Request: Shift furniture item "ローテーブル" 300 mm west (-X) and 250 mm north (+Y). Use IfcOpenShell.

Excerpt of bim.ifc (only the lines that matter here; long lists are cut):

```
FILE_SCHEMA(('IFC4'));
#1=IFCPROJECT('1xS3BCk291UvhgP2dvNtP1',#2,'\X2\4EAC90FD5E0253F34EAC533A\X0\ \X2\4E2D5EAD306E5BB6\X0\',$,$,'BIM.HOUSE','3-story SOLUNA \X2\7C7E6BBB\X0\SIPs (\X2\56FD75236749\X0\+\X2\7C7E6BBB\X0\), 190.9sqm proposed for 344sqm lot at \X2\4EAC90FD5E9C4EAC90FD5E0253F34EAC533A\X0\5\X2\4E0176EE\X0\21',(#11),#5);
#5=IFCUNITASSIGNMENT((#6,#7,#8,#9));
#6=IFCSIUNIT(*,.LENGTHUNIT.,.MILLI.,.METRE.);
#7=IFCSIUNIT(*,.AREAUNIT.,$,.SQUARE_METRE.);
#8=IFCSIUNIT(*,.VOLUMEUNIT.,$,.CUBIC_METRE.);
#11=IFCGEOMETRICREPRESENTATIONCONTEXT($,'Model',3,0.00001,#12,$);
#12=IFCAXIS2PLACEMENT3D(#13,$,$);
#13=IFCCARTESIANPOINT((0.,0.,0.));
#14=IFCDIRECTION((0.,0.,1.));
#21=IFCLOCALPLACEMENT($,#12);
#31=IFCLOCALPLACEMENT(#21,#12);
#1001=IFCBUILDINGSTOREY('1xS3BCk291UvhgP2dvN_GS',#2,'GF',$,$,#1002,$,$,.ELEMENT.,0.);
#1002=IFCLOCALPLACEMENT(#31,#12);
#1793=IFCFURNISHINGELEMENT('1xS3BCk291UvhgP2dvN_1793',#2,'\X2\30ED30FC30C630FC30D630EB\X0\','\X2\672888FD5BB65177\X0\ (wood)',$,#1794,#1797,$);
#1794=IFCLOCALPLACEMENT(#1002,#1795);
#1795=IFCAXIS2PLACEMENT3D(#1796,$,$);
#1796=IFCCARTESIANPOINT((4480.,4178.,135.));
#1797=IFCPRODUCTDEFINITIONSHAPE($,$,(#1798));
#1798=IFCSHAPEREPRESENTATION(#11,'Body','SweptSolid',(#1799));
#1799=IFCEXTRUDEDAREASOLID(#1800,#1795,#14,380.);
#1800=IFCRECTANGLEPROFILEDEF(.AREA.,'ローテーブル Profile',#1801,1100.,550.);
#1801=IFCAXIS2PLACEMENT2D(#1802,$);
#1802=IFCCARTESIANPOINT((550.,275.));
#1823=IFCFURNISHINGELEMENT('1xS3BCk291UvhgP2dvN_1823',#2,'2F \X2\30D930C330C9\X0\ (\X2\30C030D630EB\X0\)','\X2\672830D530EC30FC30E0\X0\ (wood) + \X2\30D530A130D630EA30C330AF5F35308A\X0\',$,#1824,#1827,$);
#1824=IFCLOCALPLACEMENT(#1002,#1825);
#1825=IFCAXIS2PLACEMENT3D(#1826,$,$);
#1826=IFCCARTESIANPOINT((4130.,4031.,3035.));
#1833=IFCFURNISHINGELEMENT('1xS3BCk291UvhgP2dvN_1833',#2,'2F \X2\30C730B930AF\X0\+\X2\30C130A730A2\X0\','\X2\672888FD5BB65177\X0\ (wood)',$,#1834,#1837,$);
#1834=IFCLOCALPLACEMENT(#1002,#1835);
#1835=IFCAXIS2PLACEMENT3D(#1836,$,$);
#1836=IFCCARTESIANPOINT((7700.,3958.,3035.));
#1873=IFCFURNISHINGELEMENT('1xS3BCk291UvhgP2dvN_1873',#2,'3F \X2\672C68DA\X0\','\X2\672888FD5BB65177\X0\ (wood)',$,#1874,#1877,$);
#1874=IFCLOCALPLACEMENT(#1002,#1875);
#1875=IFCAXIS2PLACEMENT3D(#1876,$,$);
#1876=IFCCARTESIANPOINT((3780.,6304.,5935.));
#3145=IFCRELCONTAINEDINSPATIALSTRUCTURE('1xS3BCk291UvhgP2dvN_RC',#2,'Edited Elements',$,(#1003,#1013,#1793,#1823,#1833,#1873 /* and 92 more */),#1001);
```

```python
import ifcopenshell
import ifcopenshell.api.geometry
import ifcopenshell.util.placement
import ifcopenshell.util.unit

model = ifcopenshell.open("bim.ifc")
unit_scale = ifcopenshell.util.unit.calculate_unit_scale(model)

item = model.by_guid("1xS3BCk291UvhgP2dvN_1793")
matrix = ifcopenshell.util.placement.get_local_placement(item.ObjectPlacement)
matrix[0, 3] -= 0.3 / unit_scale
matrix[1, 3] += 0.25 / unit_scale
ifcopenshell.api.geometry.edit_object_placement(model, product=item, matrix=matrix, is_si=False)

print(ifcopenshell.util.placement.get_local_placement(item.ObjectPlacement).round(3) + 0.0)

model.write("bim_v2.ifc")
```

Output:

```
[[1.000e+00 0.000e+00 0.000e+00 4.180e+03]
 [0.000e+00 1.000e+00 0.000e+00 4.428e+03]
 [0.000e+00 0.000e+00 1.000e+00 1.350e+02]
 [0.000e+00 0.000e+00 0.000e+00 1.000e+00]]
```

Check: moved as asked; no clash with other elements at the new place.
